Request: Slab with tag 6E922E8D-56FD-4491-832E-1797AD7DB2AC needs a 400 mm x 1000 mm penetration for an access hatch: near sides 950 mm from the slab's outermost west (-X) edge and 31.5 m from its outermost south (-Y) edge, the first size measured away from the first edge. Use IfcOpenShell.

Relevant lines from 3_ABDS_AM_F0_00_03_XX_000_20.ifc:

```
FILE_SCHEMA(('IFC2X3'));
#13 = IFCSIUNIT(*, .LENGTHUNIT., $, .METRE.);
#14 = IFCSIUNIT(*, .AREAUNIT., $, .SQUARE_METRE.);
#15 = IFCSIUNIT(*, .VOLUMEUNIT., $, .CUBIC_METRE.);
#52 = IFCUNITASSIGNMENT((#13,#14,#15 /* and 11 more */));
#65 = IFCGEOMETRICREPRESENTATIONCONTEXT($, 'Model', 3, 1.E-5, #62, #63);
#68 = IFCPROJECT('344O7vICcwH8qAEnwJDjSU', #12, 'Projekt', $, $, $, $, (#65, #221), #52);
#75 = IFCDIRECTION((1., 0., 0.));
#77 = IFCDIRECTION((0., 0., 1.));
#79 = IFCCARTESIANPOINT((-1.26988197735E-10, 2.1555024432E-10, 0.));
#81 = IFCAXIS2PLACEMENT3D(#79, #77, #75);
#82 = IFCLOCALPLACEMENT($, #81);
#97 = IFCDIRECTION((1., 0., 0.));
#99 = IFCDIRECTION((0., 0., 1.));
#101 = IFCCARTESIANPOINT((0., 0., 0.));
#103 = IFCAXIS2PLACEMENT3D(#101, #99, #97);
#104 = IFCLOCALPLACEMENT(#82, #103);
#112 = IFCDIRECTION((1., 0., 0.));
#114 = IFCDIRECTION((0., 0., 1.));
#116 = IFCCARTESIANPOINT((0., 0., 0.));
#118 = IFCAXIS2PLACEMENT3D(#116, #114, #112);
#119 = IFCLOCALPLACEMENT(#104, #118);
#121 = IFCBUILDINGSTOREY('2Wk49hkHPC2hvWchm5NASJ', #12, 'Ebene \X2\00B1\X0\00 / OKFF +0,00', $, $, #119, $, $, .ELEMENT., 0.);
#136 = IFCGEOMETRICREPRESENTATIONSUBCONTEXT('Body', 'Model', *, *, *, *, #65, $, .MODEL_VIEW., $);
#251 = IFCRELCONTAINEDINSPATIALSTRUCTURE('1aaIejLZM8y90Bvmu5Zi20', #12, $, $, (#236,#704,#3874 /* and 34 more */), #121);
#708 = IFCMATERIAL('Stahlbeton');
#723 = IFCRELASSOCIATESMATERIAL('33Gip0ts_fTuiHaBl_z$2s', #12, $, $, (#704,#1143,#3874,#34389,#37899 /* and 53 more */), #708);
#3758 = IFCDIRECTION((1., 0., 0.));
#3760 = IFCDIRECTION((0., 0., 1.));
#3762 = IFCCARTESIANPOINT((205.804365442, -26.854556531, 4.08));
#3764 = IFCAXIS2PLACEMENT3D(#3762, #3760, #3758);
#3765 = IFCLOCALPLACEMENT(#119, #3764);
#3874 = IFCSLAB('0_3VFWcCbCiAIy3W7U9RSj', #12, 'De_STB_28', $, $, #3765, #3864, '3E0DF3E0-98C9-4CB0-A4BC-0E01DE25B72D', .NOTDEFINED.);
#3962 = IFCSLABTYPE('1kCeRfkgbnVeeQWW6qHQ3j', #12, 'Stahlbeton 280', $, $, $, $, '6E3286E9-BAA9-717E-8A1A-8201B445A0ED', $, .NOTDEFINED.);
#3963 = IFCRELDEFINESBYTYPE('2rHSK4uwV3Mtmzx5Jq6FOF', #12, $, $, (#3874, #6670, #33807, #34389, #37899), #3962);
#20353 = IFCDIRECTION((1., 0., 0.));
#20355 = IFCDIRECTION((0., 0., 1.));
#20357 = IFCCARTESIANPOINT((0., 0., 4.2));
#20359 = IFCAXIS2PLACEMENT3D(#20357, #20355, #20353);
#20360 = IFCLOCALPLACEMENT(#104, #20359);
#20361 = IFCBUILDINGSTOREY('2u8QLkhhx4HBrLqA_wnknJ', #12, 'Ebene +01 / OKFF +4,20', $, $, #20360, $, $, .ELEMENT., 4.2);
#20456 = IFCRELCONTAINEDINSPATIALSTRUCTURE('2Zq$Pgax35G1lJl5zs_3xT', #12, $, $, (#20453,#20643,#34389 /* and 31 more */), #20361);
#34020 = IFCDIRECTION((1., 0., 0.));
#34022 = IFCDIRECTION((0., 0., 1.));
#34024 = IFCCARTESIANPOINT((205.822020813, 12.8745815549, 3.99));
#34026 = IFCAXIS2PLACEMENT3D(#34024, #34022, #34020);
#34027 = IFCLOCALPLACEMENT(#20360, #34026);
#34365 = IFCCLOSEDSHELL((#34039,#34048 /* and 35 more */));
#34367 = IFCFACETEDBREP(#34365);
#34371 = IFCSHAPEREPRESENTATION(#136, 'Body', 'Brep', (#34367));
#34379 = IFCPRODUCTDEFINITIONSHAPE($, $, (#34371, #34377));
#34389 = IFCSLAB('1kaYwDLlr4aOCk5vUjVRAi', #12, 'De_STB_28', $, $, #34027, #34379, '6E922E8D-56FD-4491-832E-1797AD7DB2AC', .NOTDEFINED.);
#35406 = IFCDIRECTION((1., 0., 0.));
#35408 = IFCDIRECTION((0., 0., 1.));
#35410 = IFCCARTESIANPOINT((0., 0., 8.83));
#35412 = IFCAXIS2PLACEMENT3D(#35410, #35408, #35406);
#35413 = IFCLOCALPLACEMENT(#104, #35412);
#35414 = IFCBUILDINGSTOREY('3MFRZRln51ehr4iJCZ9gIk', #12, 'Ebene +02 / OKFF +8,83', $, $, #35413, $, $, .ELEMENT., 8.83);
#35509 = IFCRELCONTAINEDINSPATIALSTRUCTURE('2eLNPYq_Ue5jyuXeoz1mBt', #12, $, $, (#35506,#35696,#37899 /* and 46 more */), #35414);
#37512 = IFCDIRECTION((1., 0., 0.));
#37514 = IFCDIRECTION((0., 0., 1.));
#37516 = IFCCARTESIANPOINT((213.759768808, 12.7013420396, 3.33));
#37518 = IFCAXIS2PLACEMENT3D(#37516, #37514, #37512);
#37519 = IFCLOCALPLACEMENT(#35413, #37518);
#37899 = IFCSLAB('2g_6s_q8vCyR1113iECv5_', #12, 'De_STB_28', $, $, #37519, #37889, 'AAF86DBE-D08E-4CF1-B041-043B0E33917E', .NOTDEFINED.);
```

```python
import numpy as np
import ifcopenshell
import ifcopenshell.api.feature
import ifcopenshell.api.geometry
import ifcopenshell.api.root
import ifcopenshell.geom
import ifcopenshell.util.placement
import ifcopenshell.util.representation
import ifcopenshell.util.shape
import ifcopenshell.util.unit

model = ifcopenshell.open("3_ABDS_AM_F0_00_03_XX_000_20.ifc")
unit_scale = ifcopenshell.util.unit.calculate_unit_scale(model)
settings = ifcopenshell.geom.settings()


def volume(element):
    """Net volume in cubic metres, openings subtracted."""
    shape = ifcopenshell.geom.create_shape(settings, element)
    return ifcopenshell.util.shape.get_volume(shape.geometry)


slab = model.by_guid("1kaYwDLlr4aOCk5vUjVRAi")
before = volume(slab)

# Extent in the slab's own axes, in metres. The edges named are its -X and -Y sides.
slab_shape = ifcopenshell.geom.create_shape(settings, slab)
vertices = ifcopenshell.util.shape.get_vertices(slab_shape.geometry)
x_min, y_min, bottom = vertices.min(axis=0)
top = vertices[:, 2].max()

opening = ifcopenshell.api.root.create_entity(model, ifc_class="IfcOpeningElement", name="Access hatch opening")
context = ifcopenshell.util.representation.get_context(model, "Model", "Body", "MODEL_VIEW")
width, depth = 0.4, 1
outline = [(0.0, 0.0), (width, 0.0), (width, depth), (0.0, depth), (0.0, 0.0)]
# Overshoot both faces by 50 mm so the cut is clean.
shape = ifcopenshell.api.geometry.add_slab_representation(
    model, context=context, depth=top - bottom + 0.1, polyline=outline
)
ifcopenshell.api.geometry.assign_representation(model, product=opening, representation=shape)

matrix = ifcopenshell.util.placement.get_local_placement(slab.ObjectPlacement)
matrix[:, 3] = matrix @ np.append(np.array([x_min + 0.95, y_min + 31.5, bottom - 0.05]) / unit_scale, 1.0)
ifcopenshell.api.geometry.edit_object_placement(model, product=opening, matrix=matrix, is_si=False)
ifcopenshell.api.feature.add_feature(model, feature=opening, element=slab)

after = volume(slab)

print(f"slab volume {before:.3f} -> {after:.3f} m3")

model.write("3_ABDS_AM_F0_00_03_XX_000_20_v2.ifc")
```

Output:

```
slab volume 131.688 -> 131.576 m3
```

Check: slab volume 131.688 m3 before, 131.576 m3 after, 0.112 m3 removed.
